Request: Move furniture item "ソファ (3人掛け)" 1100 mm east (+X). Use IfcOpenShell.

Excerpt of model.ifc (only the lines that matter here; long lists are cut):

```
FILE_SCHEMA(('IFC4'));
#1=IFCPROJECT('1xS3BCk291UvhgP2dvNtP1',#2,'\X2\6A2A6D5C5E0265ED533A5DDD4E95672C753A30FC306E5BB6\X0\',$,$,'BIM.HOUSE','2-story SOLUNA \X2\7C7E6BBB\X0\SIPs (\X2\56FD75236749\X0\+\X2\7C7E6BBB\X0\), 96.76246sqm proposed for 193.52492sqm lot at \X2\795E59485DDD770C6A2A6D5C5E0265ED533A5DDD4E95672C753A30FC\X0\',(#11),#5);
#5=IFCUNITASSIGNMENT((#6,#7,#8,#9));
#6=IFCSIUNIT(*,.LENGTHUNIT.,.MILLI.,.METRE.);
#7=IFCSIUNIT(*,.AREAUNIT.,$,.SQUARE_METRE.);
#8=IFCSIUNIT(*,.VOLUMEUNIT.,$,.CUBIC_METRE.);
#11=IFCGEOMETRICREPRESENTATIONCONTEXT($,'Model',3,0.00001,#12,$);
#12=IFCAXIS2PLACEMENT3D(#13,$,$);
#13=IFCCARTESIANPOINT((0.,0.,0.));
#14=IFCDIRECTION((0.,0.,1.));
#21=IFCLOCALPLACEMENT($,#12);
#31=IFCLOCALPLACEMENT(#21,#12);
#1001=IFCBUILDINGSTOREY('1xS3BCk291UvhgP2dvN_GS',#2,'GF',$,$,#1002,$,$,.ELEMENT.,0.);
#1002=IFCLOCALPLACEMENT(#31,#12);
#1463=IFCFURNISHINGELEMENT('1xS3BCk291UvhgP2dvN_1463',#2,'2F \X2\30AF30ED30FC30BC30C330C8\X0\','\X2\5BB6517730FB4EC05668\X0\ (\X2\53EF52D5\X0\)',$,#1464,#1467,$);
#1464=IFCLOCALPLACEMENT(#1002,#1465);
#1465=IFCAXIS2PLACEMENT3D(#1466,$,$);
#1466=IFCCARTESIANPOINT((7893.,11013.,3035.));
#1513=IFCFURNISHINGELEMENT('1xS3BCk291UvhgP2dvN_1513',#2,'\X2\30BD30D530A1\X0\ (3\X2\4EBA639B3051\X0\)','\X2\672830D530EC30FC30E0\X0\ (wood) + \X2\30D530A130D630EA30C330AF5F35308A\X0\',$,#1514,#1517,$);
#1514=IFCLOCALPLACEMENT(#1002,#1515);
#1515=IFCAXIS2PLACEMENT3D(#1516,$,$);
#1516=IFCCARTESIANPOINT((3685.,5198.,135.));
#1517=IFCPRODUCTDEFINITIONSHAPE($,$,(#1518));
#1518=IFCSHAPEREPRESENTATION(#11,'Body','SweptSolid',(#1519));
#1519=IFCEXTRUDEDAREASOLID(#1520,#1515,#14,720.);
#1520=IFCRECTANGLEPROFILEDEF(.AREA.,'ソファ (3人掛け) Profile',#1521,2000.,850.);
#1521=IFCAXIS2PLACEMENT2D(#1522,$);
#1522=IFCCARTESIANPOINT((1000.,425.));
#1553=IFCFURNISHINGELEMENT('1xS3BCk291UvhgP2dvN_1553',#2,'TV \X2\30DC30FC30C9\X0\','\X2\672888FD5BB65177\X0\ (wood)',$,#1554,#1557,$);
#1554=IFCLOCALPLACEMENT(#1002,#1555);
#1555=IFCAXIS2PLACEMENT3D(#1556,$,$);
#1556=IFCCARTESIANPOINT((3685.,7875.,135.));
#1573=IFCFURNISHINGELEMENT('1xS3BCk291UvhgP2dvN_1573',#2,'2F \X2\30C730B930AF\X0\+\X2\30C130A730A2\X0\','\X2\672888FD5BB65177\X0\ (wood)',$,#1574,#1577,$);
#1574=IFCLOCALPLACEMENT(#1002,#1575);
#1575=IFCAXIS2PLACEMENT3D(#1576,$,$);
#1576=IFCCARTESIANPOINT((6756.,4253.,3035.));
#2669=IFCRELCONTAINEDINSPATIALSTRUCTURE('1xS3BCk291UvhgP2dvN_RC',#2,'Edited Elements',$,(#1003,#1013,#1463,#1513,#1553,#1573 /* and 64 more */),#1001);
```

```python
import ifcopenshell
import ifcopenshell.api.geometry
import ifcopenshell.util.placement

model = ifcopenshell.open("model.ifc")

item = model.by_guid("1xS3BCk291UvhgP2dvN_1513")
matrix = ifcopenshell.util.placement.get_local_placement(item.ObjectPlacement)
matrix[0, 3] += 1100.0
ifcopenshell.api.geometry.edit_object_placement(model, product=item, matrix=matrix, is_si=False)

print(ifcopenshell.util.placement.get_local_placement(item.ObjectPlacement).round(3) + 0.0)

model.write("model_updated.ifc")
```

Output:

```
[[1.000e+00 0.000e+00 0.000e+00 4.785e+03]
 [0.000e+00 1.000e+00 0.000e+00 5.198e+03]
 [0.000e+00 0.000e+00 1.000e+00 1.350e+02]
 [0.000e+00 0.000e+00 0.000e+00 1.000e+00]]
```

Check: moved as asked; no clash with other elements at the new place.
